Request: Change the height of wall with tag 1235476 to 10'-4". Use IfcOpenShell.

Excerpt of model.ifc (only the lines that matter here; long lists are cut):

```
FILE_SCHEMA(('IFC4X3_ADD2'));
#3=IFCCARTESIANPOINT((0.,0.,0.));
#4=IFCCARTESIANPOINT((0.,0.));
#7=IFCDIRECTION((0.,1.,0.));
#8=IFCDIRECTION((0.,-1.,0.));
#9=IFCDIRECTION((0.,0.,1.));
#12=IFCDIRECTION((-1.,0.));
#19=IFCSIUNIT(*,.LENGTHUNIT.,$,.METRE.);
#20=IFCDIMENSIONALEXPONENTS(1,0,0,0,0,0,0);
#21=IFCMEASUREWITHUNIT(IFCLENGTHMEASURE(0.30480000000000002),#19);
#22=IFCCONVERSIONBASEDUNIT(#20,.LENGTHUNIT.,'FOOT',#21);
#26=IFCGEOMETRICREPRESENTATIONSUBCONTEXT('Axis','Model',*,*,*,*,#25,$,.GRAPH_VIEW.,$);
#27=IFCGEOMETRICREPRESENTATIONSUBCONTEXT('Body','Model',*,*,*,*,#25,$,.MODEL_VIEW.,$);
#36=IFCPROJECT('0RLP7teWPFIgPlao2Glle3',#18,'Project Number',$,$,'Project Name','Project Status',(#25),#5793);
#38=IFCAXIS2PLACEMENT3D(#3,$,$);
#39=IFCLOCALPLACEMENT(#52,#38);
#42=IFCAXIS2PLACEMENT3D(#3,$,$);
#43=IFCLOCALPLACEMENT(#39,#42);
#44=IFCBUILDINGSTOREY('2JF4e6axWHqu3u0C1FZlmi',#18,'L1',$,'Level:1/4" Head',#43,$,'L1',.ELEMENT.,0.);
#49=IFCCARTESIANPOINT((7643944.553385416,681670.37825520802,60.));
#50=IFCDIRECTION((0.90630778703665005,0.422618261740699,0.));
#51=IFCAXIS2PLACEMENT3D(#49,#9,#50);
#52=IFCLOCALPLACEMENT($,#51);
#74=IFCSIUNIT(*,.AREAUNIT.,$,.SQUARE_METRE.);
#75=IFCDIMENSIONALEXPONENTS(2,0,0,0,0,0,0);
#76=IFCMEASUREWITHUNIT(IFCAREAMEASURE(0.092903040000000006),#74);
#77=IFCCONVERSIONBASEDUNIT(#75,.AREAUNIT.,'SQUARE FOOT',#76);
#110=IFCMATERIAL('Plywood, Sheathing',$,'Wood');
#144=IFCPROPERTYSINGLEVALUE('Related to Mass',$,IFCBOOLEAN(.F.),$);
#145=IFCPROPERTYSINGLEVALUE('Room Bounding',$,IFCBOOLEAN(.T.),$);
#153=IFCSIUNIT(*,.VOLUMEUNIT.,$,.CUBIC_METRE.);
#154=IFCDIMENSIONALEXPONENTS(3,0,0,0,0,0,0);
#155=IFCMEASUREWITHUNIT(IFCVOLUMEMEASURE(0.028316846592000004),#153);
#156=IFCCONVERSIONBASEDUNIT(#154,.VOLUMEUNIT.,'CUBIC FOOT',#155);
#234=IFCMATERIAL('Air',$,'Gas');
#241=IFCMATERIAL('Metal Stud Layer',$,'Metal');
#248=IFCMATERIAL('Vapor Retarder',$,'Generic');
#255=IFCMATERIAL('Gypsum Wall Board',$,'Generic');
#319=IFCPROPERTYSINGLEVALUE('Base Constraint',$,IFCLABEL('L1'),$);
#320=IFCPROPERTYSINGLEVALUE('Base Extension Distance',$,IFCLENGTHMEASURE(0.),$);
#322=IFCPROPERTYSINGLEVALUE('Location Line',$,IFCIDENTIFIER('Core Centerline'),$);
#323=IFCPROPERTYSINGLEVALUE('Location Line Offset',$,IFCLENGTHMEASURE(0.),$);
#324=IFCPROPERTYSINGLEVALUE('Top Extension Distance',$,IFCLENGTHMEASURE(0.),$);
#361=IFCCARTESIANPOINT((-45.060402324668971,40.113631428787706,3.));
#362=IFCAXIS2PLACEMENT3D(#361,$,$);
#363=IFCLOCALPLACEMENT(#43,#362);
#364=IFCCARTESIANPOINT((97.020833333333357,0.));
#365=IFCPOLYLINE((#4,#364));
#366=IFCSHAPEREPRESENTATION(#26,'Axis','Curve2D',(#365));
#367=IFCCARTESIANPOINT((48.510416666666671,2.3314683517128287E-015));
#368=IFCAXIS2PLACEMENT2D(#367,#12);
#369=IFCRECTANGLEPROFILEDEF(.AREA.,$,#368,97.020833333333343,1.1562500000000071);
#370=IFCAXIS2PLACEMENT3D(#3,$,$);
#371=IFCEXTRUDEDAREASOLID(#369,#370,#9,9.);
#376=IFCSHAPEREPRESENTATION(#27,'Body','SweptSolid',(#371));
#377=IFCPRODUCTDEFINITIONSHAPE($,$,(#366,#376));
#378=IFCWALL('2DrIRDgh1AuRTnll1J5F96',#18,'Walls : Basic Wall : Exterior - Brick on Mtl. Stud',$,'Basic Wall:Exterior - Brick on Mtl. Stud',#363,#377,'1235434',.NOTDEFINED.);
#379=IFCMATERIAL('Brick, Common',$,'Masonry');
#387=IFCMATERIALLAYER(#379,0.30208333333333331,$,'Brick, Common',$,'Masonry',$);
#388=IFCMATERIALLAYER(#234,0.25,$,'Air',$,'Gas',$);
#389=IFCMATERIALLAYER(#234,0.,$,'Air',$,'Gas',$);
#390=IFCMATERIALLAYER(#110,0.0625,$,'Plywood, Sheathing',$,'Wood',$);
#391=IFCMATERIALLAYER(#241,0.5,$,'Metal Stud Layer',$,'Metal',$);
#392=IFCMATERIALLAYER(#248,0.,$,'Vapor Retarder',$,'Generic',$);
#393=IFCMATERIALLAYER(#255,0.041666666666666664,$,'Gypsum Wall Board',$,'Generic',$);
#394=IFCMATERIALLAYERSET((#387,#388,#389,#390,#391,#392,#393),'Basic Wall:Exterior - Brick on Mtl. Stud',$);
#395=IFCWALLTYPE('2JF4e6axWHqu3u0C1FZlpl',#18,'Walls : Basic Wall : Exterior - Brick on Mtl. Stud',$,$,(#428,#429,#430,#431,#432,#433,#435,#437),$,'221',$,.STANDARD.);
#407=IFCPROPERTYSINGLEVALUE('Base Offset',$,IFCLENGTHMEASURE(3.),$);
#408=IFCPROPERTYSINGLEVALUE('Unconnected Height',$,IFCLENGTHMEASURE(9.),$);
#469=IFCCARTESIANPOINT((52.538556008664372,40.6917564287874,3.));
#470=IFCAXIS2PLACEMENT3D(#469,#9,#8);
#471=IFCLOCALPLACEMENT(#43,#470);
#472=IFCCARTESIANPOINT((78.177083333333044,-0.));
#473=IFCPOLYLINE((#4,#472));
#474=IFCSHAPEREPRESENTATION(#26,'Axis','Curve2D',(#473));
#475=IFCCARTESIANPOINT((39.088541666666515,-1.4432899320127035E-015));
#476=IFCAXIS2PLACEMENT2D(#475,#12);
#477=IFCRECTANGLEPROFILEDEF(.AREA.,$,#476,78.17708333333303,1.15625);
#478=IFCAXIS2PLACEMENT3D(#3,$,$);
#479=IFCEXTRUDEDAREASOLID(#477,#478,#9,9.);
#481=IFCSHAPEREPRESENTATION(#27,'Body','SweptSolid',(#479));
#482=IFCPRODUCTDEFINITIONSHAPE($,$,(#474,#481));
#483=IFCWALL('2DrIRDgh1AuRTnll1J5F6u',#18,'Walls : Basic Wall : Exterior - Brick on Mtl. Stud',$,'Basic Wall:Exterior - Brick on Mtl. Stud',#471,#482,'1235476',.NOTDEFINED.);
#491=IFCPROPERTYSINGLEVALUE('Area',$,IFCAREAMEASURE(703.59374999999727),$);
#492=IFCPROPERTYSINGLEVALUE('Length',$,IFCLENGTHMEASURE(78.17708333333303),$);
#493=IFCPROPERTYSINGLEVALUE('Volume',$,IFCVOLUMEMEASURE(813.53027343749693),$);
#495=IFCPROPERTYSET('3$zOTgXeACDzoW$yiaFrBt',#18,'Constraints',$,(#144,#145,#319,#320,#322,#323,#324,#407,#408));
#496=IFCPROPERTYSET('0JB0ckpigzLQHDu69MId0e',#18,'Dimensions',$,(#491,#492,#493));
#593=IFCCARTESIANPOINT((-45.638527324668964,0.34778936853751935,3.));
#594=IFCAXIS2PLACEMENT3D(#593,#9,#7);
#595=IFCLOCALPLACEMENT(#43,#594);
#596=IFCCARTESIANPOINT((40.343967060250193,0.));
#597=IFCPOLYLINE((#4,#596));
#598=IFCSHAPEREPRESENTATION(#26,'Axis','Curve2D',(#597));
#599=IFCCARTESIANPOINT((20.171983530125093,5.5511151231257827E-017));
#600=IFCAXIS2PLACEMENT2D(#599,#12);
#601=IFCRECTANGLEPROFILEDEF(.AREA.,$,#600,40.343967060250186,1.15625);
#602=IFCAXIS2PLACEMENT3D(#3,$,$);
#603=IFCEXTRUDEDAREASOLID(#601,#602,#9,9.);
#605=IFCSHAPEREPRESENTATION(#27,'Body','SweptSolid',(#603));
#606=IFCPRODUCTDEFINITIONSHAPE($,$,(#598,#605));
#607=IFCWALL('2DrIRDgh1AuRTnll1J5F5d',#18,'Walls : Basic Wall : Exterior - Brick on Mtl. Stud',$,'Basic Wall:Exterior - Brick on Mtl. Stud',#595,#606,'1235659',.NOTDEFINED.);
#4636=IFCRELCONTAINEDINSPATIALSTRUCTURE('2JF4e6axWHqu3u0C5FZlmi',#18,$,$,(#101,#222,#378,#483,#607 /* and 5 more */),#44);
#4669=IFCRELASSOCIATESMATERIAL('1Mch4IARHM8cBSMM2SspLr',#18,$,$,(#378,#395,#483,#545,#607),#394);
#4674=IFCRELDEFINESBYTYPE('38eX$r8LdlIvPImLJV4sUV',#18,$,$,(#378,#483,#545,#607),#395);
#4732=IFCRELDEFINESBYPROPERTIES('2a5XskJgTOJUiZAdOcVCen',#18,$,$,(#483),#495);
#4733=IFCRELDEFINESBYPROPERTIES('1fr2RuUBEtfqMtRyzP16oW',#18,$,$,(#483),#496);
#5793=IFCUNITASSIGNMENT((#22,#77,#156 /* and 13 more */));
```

```python
import ifcopenshell
import ifcopenshell.api.pset
import ifcopenshell.geom
import ifcopenshell.util.element
import ifcopenshell.util.representation
import ifcopenshell.util.shape
import ifcopenshell.util.unit

model = ifcopenshell.open("model.ifc")
unit_scale = ifcopenshell.util.unit.calculate_unit_scale(model)
area_scale = ifcopenshell.util.unit.calculate_unit_scale(model, "AREAUNIT")
volume_scale = ifcopenshell.util.unit.calculate_unit_scale(model, "VOLUMEUNIT")
settings = ifcopenshell.geom.settings()


def volume(element):
    """Net volume in cubic metres, openings subtracted."""
    shape = ifcopenshell.geom.create_shape(settings, element)
    return ifcopenshell.util.shape.get_volume(shape.geometry)


wall = model.by_id(483)
before = volume(wall)

body = ifcopenshell.util.representation.get_representation(wall, "Model", "Body")
solid = body.Items[0]
old_height = solid.Depth
solid.Depth = 124 * 0.0254 / unit_scale
after = volume(wall)
thickness = 0.3524  # wall thickness in metres

# Update the stored height, areas and volumes.
pset = model.by_id(ifcopenshell.util.element.get_pset(wall, "Constraints", should_inherit=False)["id"])
ifcopenshell.api.pset.edit_pset(model, pset=pset, properties={
    "Unconnected Height": model.create_entity("IfcLengthMeasure", solid.Depth),
})
pset = model.by_id(ifcopenshell.util.element.get_pset(wall, "Dimensions", should_inherit=False)["id"])
ifcopenshell.api.pset.edit_pset(model, pset=pset, properties={
    "Area": model.create_entity("IfcAreaMeasure", after / thickness / area_scale),
    "Volume": model.create_entity("IfcVolumeMeasure", after / volume_scale),
})

print(f"height {old_height:g} -> {solid.Depth:g}, volume {before:.3f} -> {after:.3f} m3")

model.write("model_edited.ifc")
```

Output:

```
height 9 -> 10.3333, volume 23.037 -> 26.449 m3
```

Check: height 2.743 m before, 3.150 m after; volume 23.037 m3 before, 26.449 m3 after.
